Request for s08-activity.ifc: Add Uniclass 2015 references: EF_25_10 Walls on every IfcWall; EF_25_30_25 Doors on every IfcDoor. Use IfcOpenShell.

First a look at what the model holds.

```python
import ifcopenshell

model = ifcopenshell.open("s08-activity.ifc")
print(model.schema)
print("classifications:", [c.Name for c in model.by_type("IfcClassification")])
for ifc_class in ("IfcDoor", "IfcRoof", "IfcStair", "IfcWall", "IfcWindow"):
    print(ifc_class, len(model.by_type(ifc_class)))
```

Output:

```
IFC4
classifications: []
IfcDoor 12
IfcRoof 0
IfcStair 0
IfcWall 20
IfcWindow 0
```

```python
import ifcopenshell
import ifcopenshell.api.classification

model = ifcopenshell.open("s08-activity.ifc")

system = ifcopenshell.api.classification.add_classification(model, classification="Uniclass 2015")

codes = {
    "IfcWall": ("EF_25_10", "Walls"),
    "IfcDoor": ("EF_25_30_25", "Doors"),
}
for ifc_class, (code, name) in codes.items():
    products = model.by_type(ifc_class)
    ifcopenshell.api.classification.add_reference(
        model, products=products, classification=system, identification=code, name=name
    )
    print(code, len(products))

model.write("s08-activity_updated.ifc")
```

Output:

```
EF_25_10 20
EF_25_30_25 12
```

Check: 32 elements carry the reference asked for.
